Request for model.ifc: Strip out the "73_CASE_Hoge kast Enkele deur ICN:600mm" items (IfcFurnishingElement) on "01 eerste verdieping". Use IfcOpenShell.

First a look at what the model holds.

```python
import ifcopenshell
import ifcopenshell.util.element

model = ifcopenshell.open("model.ifc")
print(model.schema)
storey = next(s for s in model.by_type("IfcBuildingStorey") if s.Name == "01 eerste verdieping")
furniture = [e for e in ifcopenshell.util.element.get_decomposition(storey) if e.is_a("IfcFurnishingElement")]
seen = {}
for e in furniture:
    element_type = ifcopenshell.util.element.get_type(e)
    name = element_type.Name if element_type not in (None, e) else None
    seen[name] = seen.get(name, 0) + 1
for name, count in sorted(seen.items(), key=str):
    print(count, "x", name)
```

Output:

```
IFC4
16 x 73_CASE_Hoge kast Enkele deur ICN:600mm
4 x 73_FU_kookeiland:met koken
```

```python
import ifcopenshell
import ifcopenshell.api.root
import ifcopenshell.util.element

model = ifcopenshell.open("model.ifc")

storey = next(s for s in model.by_type("IfcBuildingStorey") if s.Name == "01 eerste verdieping")
furniture = [e for e in ifcopenshell.util.element.get_decomposition(storey) if e.is_a("IfcFurnishingElement")]
targets = [e for e in furniture if (t := ifcopenshell.util.element.get_type(e)) not in (None, e) and t.Name == "73_CASE_Hoge kast Enkele deur ICN:600mm"]

for e in targets:
    ifcopenshell.api.root.remove_product(model, product=e)
print(len(targets), "removed")

model.write("model_updated.ifc")
```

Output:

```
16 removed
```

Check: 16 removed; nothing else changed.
